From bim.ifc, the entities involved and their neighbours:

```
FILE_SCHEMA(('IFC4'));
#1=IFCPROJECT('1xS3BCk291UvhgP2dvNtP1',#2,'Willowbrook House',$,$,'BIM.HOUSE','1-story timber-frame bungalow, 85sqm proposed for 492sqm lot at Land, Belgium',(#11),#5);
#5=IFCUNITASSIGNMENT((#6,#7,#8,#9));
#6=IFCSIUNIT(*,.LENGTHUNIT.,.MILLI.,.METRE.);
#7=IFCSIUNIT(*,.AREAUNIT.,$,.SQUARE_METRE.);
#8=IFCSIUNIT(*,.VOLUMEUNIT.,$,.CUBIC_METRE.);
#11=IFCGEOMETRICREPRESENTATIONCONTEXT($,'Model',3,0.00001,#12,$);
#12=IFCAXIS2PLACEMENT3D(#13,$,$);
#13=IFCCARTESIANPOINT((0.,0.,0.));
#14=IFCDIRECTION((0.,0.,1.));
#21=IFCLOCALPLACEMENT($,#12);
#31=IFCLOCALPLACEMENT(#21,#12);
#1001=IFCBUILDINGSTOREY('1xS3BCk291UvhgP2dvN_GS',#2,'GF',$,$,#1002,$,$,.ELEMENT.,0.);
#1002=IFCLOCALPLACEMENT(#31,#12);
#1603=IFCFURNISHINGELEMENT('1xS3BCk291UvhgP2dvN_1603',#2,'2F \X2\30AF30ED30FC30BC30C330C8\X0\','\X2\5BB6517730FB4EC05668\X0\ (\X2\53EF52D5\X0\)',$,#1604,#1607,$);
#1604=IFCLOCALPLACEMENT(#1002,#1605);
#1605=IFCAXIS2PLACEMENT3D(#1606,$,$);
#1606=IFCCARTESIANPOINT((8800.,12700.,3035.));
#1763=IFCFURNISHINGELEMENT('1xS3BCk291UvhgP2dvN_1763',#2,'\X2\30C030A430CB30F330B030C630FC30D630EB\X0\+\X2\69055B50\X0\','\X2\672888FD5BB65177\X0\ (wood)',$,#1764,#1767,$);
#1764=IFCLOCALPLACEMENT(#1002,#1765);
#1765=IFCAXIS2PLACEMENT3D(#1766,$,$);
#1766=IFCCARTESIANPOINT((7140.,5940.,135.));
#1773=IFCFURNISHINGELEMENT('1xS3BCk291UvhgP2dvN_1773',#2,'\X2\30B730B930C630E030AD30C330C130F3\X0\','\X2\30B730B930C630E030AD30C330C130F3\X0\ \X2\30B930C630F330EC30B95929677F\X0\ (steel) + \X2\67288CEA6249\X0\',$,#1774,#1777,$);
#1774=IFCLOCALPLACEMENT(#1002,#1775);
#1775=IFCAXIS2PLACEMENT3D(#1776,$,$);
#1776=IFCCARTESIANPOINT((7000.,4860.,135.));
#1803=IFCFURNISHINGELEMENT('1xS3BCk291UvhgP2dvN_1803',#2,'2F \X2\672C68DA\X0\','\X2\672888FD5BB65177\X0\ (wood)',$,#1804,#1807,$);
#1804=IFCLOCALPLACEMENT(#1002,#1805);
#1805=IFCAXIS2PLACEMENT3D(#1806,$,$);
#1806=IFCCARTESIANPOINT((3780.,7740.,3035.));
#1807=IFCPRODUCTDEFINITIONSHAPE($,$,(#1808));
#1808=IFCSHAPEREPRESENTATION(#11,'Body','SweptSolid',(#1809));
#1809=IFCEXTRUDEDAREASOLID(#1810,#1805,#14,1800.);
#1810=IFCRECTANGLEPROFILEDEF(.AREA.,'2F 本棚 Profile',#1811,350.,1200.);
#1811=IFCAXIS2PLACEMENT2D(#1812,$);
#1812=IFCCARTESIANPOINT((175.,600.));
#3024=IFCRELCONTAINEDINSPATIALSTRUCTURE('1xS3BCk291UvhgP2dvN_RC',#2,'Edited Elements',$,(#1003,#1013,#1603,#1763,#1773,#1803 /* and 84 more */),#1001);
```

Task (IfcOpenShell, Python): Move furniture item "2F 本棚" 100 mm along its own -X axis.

```python
import ifcopenshell
import ifcopenshell.api.geometry
import ifcopenshell.util.placement
import ifcopenshell.util.unit

model = ifcopenshell.open("bim.ifc")
unit_scale = ifcopenshell.util.unit.calculate_unit_scale(model)

item = model.by_id(1803)
matrix = ifcopenshell.util.placement.get_local_placement(item.ObjectPlacement)
matrix[:3, 3] -= matrix[:3, 0] * 0.1 / unit_scale
ifcopenshell.api.geometry.edit_object_placement(model, product=item, matrix=matrix, is_si=False)

print(ifcopenshell.util.placement.get_local_placement(item.ObjectPlacement).round(3) + 0.0)

model.write("bim-out.ifc")
```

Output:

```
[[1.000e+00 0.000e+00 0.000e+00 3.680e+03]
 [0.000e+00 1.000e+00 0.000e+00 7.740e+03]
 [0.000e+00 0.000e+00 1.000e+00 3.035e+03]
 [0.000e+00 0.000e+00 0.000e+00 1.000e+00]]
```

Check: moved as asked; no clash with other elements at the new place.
